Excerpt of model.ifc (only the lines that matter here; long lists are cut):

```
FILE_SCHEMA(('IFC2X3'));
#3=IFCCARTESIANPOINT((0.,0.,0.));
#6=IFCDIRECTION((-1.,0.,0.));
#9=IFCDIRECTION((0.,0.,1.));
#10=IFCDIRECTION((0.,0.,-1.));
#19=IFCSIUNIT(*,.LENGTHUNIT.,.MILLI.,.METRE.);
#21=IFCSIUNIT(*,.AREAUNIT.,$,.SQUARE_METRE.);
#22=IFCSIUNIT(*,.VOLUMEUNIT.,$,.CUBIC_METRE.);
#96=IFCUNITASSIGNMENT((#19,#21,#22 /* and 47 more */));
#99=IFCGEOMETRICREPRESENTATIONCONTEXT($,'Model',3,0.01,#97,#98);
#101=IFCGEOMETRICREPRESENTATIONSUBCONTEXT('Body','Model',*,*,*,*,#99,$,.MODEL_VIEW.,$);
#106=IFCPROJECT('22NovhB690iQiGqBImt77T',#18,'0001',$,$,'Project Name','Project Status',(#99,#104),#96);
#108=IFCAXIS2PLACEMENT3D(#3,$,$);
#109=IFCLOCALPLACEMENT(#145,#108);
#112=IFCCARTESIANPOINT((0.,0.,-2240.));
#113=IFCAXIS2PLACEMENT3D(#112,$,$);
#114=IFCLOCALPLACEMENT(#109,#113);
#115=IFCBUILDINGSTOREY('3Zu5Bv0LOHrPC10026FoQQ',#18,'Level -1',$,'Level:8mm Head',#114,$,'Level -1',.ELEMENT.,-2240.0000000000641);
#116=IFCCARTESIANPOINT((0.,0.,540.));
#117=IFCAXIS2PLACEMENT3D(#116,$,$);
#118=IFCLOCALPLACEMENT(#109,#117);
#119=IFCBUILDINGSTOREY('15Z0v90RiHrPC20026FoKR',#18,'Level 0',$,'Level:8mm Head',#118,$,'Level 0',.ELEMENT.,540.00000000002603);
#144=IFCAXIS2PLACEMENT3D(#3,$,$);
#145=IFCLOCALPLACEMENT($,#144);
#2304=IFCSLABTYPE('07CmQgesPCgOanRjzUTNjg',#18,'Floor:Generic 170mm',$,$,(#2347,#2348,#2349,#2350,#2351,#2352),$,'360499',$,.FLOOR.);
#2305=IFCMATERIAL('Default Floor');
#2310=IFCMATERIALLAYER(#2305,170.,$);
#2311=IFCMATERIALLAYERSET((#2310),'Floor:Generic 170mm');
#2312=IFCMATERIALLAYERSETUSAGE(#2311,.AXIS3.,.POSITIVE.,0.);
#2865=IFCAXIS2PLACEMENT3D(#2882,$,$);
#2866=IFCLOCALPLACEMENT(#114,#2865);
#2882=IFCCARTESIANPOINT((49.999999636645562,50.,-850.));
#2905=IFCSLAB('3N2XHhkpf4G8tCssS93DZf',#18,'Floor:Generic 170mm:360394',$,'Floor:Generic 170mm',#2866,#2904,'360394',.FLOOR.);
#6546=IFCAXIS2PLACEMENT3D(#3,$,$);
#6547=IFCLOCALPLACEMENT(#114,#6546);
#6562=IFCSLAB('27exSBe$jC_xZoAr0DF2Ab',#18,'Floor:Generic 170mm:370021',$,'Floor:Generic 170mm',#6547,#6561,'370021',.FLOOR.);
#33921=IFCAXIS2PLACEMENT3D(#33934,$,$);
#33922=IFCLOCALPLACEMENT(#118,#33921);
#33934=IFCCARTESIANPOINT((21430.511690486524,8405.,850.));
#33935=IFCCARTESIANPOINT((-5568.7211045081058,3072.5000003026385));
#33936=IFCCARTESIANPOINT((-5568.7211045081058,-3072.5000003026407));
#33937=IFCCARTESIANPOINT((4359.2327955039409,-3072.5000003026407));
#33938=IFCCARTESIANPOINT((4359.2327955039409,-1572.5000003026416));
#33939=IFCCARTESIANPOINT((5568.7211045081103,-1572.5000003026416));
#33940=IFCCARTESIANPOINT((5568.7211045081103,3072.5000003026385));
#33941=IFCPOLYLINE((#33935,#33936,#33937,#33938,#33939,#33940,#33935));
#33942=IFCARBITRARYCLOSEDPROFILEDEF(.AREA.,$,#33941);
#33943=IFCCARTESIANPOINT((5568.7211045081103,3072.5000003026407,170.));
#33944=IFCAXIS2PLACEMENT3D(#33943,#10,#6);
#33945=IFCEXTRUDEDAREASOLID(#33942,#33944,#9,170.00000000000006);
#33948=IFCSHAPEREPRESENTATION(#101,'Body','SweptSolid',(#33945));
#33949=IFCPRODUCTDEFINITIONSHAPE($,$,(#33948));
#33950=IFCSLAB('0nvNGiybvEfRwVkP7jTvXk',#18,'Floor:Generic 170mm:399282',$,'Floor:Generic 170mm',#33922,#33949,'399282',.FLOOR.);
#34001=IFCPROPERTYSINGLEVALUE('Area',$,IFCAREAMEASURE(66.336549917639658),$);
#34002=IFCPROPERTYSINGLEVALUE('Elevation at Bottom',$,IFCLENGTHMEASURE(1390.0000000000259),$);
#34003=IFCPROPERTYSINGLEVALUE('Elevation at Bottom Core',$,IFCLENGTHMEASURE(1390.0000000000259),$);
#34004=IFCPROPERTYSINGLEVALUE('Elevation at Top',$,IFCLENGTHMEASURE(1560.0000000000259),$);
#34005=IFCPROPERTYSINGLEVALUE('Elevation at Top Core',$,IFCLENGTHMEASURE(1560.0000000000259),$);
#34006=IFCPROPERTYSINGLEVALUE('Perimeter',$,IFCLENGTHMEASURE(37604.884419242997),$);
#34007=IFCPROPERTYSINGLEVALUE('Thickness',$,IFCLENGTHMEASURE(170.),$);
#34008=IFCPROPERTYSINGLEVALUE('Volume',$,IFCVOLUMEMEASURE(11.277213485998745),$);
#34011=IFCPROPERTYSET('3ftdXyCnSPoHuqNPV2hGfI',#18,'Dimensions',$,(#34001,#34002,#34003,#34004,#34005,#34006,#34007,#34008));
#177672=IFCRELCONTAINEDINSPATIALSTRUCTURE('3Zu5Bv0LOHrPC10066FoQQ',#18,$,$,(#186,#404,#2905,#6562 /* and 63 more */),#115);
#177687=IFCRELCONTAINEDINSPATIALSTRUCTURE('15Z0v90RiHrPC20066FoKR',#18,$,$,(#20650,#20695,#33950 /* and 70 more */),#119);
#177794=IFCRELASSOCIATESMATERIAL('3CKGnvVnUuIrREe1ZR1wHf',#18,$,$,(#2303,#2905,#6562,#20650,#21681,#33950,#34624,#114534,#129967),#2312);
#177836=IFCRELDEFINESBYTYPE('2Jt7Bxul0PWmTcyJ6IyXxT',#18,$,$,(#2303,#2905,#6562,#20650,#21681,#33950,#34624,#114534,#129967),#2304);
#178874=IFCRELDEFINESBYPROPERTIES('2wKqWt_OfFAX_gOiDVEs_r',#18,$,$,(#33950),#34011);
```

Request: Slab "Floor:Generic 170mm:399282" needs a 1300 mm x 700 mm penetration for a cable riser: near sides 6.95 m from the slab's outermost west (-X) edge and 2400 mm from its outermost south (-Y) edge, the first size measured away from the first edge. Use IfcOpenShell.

```python
import numpy as np
import ifcopenshell
import ifcopenshell.api.feature
import ifcopenshell.api.geometry
import ifcopenshell.api.pset
import ifcopenshell.api.root
import ifcopenshell.geom
import ifcopenshell.util.element
import ifcopenshell.util.placement
import ifcopenshell.util.representation
import ifcopenshell.util.shape
import ifcopenshell.util.unit

model = ifcopenshell.open("model.ifc")
unit_scale = ifcopenshell.util.unit.calculate_unit_scale(model)
area_scale = ifcopenshell.util.unit.calculate_unit_scale(model, "AREAUNIT")
volume_scale = ifcopenshell.util.unit.calculate_unit_scale(model, "VOLUMEUNIT")
settings = ifcopenshell.geom.settings()


def volume(element):
    """Net volume in cubic metres, openings subtracted."""
    shape = ifcopenshell.geom.create_shape(settings, element)
    return ifcopenshell.util.shape.get_volume(shape.geometry)


slab = model.by_guid("0nvNGiybvEfRwVkP7jTvXk")
before = volume(slab)

# Extent in the slab's own axes, in metres. The edges named are its -X and -Y sides.
slab_shape = ifcopenshell.geom.create_shape(settings, slab)
vertices = ifcopenshell.util.shape.get_vertices(slab_shape.geometry)
x_min, y_min, bottom = vertices.min(axis=0)
top = vertices[:, 2].max()

opening = ifcopenshell.api.root.create_entity(model, ifc_class="IfcOpeningElement", name="Cable riser opening")
context = ifcopenshell.util.representation.get_context(model, "Model", "Body", "MODEL_VIEW")
width, depth = 1.3, 0.7
outline = [(0.0, 0.0), (width, 0.0), (width, depth), (0.0, depth), (0.0, 0.0)]
# Overshoot both faces by 50 mm so the cut is clean.
shape = ifcopenshell.api.geometry.add_slab_representation(
    model, context=context, depth=top - bottom + 0.1, polyline=outline
)
ifcopenshell.api.geometry.assign_representation(model, product=opening, representation=shape)

matrix = ifcopenshell.util.placement.get_local_placement(slab.ObjectPlacement)
matrix[:, 3] = matrix @ np.append(np.array([x_min + 6.95, y_min + 2.4, bottom - 0.05]) / unit_scale, 1.0)
ifcopenshell.api.geometry.edit_object_placement(model, product=opening, matrix=matrix, is_si=False)
ifcopenshell.api.feature.add_feature(model, feature=opening, element=slab)

after = volume(slab)

# Update the slab's stored quantities.
pset = model.by_id(ifcopenshell.util.element.get_pset(slab, "Dimensions", should_inherit=False)["id"])
ifcopenshell.api.pset.edit_pset(model, pset=pset, properties={
    "Area": model.create_entity("IfcAreaMeasure", after / (top - bottom) / area_scale),
    "Volume": model.create_entity("IfcVolumeMeasure", after / volume_scale),
})

print(f"slab volume {before:.3f} -> {after:.3f} m3")

model.write("model_edited.ifc")
```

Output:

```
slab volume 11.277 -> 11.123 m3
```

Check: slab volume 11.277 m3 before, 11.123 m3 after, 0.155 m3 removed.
